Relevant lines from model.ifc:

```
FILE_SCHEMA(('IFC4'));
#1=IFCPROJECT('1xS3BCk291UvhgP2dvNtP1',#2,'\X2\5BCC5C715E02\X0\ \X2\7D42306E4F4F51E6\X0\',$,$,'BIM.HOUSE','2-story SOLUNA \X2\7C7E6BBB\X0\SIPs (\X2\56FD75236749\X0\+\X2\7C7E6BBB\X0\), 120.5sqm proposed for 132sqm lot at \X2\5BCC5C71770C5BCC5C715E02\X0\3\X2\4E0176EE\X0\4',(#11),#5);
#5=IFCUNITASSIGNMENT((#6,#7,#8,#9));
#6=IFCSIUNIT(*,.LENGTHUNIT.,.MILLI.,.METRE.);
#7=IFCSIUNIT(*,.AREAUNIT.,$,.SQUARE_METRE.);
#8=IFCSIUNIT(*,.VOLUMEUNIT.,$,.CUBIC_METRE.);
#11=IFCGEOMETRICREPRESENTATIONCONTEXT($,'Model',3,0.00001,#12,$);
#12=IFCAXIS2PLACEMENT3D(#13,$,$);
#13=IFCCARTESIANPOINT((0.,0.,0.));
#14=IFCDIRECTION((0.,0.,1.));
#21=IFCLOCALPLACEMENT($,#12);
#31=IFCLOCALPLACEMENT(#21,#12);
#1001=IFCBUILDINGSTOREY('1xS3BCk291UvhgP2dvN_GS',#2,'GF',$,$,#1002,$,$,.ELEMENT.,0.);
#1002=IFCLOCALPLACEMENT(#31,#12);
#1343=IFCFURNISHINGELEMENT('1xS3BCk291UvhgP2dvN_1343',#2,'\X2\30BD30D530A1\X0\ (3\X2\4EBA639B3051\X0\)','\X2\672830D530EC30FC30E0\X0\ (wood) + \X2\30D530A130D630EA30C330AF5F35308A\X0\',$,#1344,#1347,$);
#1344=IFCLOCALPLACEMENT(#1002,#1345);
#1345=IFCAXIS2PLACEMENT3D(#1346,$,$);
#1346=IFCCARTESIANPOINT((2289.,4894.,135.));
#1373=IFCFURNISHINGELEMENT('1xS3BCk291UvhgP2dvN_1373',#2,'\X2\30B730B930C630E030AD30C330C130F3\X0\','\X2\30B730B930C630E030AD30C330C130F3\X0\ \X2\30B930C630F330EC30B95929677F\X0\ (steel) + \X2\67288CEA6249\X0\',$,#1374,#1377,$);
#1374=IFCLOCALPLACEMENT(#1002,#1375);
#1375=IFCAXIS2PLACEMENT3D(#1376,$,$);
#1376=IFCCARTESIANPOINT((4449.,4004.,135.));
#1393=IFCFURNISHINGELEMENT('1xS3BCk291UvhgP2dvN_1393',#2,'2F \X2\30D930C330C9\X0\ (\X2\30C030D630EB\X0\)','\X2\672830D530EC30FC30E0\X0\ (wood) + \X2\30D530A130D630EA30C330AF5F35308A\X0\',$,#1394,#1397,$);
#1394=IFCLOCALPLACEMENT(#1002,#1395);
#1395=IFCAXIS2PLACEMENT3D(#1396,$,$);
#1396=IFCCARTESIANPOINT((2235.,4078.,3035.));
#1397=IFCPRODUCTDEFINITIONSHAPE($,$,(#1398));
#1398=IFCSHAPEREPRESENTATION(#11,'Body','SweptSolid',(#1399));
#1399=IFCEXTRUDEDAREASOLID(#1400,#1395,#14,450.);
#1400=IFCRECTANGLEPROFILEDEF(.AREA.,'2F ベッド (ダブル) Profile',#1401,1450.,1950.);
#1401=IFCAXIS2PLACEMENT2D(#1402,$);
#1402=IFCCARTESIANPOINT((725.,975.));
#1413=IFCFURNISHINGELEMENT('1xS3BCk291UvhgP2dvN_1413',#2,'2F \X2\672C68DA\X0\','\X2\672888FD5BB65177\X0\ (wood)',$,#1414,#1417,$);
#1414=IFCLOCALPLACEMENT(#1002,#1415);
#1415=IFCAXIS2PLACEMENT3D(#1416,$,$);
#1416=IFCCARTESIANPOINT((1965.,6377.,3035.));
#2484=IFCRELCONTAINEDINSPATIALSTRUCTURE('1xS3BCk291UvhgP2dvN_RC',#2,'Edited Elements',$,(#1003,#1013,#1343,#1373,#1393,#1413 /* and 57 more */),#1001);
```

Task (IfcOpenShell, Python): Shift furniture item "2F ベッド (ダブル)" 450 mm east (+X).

```python
import ifcopenshell
import ifcopenshell.api.geometry
import ifcopenshell.util.placement
import ifcopenshell.util.unit

model = ifcopenshell.open("model.ifc")
unit_scale = ifcopenshell.util.unit.calculate_unit_scale(model)

item = model.by_id(1393)
matrix = ifcopenshell.util.placement.get_local_placement(item.ObjectPlacement)
matrix[0, 3] += 0.45 / unit_scale
ifcopenshell.api.geometry.edit_object_placement(model, product=item, matrix=matrix, is_si=False)

print(ifcopenshell.util.placement.get_local_placement(item.ObjectPlacement).round(3) + 0.0)

model.write("model_edited.ifc")
```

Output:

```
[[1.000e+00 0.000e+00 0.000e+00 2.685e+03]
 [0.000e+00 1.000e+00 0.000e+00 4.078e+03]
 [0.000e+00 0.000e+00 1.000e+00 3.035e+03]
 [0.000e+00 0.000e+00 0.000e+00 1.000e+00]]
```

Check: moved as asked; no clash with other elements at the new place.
